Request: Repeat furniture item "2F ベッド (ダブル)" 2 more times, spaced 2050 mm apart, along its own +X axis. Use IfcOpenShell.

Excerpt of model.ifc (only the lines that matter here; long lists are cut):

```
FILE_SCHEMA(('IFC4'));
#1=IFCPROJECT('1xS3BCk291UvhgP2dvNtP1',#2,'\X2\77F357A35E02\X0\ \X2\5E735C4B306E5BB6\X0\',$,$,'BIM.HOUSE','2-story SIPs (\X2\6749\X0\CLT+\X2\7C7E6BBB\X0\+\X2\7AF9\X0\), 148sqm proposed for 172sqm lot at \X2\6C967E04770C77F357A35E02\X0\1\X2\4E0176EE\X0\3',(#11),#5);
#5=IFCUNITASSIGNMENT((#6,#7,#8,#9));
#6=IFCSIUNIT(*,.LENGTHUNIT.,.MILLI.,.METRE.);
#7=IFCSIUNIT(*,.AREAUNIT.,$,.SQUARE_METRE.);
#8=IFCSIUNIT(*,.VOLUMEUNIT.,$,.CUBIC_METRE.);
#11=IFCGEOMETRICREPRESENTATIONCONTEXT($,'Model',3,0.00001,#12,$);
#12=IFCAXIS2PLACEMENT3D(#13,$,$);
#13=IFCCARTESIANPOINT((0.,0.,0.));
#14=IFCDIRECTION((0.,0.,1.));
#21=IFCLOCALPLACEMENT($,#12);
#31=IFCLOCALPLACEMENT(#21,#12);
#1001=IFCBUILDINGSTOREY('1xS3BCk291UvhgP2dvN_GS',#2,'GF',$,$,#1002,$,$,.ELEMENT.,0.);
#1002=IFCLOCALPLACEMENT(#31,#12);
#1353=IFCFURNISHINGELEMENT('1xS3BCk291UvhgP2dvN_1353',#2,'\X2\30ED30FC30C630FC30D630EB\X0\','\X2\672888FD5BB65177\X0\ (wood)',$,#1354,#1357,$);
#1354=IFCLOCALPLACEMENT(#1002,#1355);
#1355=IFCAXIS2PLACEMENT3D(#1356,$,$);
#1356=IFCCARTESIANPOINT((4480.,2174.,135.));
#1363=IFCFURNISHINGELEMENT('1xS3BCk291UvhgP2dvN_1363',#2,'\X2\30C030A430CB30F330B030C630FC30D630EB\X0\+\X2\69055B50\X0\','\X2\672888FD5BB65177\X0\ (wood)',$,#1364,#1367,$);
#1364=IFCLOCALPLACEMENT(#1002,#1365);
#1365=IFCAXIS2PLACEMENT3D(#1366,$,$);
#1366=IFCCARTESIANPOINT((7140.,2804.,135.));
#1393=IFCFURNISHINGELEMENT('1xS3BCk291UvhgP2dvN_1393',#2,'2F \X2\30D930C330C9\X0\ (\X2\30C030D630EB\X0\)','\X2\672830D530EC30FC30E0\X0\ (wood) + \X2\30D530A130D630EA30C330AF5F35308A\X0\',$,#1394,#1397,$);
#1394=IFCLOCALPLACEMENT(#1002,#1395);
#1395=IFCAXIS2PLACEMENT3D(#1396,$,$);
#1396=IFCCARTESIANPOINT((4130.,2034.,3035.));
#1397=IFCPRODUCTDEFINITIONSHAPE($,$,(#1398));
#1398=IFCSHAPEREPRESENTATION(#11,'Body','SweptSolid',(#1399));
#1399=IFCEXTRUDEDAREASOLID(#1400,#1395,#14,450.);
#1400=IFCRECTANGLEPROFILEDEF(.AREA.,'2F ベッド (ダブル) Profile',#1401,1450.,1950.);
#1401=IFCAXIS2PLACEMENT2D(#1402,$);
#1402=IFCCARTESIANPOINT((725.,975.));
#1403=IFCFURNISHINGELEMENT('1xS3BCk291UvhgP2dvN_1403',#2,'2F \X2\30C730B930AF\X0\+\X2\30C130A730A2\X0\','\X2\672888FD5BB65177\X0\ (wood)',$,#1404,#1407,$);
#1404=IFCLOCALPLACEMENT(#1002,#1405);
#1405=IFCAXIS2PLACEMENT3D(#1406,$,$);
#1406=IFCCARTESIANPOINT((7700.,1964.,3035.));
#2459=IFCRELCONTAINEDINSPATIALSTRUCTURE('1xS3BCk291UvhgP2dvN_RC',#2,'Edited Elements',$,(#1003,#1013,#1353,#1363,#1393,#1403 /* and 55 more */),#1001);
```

```python
import ifcopenshell
import ifcopenshell.api.geometry
import ifcopenshell.api.root
import ifcopenshell.util.element
import ifcopenshell.util.placement

model = ifcopenshell.open("model.ifc")


def reuse_history(source, copy):
    """copy_class also copies each property set's owner history, people and application; keep the originals."""
    for rel in copy.IsDefinedBy:
        if rel.is_a("IfcRelDefinesByProperties") and (history := rel.RelatingPropertyDefinition.OwnerHistory):
            rel.RelatingPropertyDefinition.OwnerHistory = source.OwnerHistory
            ifcopenshell.util.element.remove_deep2(model, history)


source = model.by_id(1393)
base = ifcopenshell.util.placement.get_local_placement(source.ObjectPlacement)
step = base[:3, 0] * 2050.0

for i in range(1, 3):
    copy = ifcopenshell.api.root.copy_class(model, product=source)
    copy.Representation = ifcopenshell.util.element.copy_deep(
        model, source.Representation, exclude=["IfcGeometricRepresentationContext", "IfcRepresentationMap"]
    )
    reuse_history(source, copy)
    matrix = base.copy()
    matrix[:3, 3] += i * step
    print("added at", matrix[:3, 3].round(3) + 0.0)
    ifcopenshell.api.geometry.edit_object_placement(model, product=copy, matrix=matrix, is_si=False)

model.write("model_v2.ifc")
```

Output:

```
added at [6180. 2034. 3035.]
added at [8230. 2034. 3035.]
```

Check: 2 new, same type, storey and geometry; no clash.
